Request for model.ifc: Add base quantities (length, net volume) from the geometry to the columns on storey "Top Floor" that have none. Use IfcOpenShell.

First a look at what the model holds.

```python
import ifcopenshell
import ifcopenshell.util.element
import ifcopenshell.util.unit

model = ifcopenshell.open("model.ifc")
print(model.schema)
for unit_type in ("LENGTHUNIT", "AREAUNIT", "VOLUMEUNIT"):
    print(unit_type, ifcopenshell.util.unit.calculate_unit_scale(model, unit_type))
storey = next(s for s in model.by_type("IfcBuildingStorey") if s.Name == "Top Floor")
columns = [e for e in ifcopenshell.util.element.get_decomposition(storey) if e.is_a("IfcColumn")]
for e in sorted(columns, key=lambda e: e.id()):
    print(e.id(), e.is_a(), e.Name, list(ifcopenshell.util.element.get_psets(e, qtos_only=True)), sep=" | ")
```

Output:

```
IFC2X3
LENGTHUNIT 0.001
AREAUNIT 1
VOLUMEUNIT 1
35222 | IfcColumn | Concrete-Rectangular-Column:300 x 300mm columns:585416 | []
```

```python
import ifcopenshell
import ifcopenshell.api.pset
import ifcopenshell.geom
import ifcopenshell.util.element
import ifcopenshell.util.shape
import ifcopenshell.util.unit

model = ifcopenshell.open("model.ifc")
unit_scale = ifcopenshell.util.unit.calculate_unit_scale(model)
volume_scale = ifcopenshell.util.unit.calculate_unit_scale(model, "VOLUMEUNIT")
settings = ifcopenshell.geom.settings()

storey = next(s for s in model.by_type("IfcBuildingStorey") if s.Name == "Top Floor")
columns = [e for e in ifcopenshell.util.element.get_decomposition(storey) if e.is_a("IfcColumn")]

for e in sorted(columns, key=lambda e: e.id()):
    if ifcopenshell.util.element.get_psets(e, qtos_only=True, should_inherit=False):
        continue
    # Geometry comes back in metres, in the element's own axes.
    shape = ifcopenshell.geom.create_shape(settings, e)
    values = {
        "Length": ifcopenshell.util.shape.get_z(shape.geometry) / unit_scale,
        "NetVolume": ifcopenshell.util.shape.get_volume(shape.geometry) / volume_scale,
    }
    qto = ifcopenshell.api.pset.add_qto(model, product=e, name="BaseQuantities")
    ifcopenshell.api.pset.edit_qto(model, qto=qto, properties=values)
    print(e.id(), {k: round(v, 3) for k, v in values.items()})

model.write("model_v2.ifc")
```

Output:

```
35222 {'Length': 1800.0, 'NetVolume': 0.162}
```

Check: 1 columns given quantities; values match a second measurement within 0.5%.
